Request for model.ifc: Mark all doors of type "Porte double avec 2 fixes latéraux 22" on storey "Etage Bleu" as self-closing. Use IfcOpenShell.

First a look at what the model holds.

```python
import ifcopenshell
import ifcopenshell.util.element

model = ifcopenshell.open("model.ifc")
print(model.schema)
storey = next(s for s in model.by_type("IfcBuildingStorey") if s.Name == "Etage Bleu")
doors = [e for e in ifcopenshell.util.element.get_decomposition(storey) if e.is_a("IfcDoor")]
seen = {}
for e in doors:
    element_type = ifcopenshell.util.element.get_type(e)
    key = (element_type.Name if element_type != e and element_type else None, ifcopenshell.util.element.get_pset(e, "Pset_DoorCommon", "SelfClosing"))
    seen[key] = seen.get(key, 0) + 1
for (name, value), count in sorted(seen.items(), key=str):
    print(count, "x", name, "|", value)
```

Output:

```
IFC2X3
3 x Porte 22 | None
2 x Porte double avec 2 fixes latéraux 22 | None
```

```python
import ifcopenshell
import ifcopenshell.api.pset
import ifcopenshell.util.element

model = ifcopenshell.open("model.ifc")

storey = next(s for s in model.by_type("IfcBuildingStorey") if s.Name == "Etage Bleu")
doors = [e for e in ifcopenshell.util.element.get_decomposition(storey) if e.is_a("IfcDoor")]

count = 0
for e in doors:
    element_type = ifcopenshell.util.element.get_type(e)
    if element_type in (None, e) or element_type.Name != "Porte double avec 2 fixes latéraux 22":
        continue
    # add_pset returns the element's existing set when there is one.
    pset = ifcopenshell.api.pset.add_pset(model, product=e, name="Pset_DoorCommon")
    ifcopenshell.api.pset.edit_pset(model, pset=pset, properties={"SelfClosing": True})
    count += 1

print(count, "doors updated")

model.write("model_rev.ifc")
```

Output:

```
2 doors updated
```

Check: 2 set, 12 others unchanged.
